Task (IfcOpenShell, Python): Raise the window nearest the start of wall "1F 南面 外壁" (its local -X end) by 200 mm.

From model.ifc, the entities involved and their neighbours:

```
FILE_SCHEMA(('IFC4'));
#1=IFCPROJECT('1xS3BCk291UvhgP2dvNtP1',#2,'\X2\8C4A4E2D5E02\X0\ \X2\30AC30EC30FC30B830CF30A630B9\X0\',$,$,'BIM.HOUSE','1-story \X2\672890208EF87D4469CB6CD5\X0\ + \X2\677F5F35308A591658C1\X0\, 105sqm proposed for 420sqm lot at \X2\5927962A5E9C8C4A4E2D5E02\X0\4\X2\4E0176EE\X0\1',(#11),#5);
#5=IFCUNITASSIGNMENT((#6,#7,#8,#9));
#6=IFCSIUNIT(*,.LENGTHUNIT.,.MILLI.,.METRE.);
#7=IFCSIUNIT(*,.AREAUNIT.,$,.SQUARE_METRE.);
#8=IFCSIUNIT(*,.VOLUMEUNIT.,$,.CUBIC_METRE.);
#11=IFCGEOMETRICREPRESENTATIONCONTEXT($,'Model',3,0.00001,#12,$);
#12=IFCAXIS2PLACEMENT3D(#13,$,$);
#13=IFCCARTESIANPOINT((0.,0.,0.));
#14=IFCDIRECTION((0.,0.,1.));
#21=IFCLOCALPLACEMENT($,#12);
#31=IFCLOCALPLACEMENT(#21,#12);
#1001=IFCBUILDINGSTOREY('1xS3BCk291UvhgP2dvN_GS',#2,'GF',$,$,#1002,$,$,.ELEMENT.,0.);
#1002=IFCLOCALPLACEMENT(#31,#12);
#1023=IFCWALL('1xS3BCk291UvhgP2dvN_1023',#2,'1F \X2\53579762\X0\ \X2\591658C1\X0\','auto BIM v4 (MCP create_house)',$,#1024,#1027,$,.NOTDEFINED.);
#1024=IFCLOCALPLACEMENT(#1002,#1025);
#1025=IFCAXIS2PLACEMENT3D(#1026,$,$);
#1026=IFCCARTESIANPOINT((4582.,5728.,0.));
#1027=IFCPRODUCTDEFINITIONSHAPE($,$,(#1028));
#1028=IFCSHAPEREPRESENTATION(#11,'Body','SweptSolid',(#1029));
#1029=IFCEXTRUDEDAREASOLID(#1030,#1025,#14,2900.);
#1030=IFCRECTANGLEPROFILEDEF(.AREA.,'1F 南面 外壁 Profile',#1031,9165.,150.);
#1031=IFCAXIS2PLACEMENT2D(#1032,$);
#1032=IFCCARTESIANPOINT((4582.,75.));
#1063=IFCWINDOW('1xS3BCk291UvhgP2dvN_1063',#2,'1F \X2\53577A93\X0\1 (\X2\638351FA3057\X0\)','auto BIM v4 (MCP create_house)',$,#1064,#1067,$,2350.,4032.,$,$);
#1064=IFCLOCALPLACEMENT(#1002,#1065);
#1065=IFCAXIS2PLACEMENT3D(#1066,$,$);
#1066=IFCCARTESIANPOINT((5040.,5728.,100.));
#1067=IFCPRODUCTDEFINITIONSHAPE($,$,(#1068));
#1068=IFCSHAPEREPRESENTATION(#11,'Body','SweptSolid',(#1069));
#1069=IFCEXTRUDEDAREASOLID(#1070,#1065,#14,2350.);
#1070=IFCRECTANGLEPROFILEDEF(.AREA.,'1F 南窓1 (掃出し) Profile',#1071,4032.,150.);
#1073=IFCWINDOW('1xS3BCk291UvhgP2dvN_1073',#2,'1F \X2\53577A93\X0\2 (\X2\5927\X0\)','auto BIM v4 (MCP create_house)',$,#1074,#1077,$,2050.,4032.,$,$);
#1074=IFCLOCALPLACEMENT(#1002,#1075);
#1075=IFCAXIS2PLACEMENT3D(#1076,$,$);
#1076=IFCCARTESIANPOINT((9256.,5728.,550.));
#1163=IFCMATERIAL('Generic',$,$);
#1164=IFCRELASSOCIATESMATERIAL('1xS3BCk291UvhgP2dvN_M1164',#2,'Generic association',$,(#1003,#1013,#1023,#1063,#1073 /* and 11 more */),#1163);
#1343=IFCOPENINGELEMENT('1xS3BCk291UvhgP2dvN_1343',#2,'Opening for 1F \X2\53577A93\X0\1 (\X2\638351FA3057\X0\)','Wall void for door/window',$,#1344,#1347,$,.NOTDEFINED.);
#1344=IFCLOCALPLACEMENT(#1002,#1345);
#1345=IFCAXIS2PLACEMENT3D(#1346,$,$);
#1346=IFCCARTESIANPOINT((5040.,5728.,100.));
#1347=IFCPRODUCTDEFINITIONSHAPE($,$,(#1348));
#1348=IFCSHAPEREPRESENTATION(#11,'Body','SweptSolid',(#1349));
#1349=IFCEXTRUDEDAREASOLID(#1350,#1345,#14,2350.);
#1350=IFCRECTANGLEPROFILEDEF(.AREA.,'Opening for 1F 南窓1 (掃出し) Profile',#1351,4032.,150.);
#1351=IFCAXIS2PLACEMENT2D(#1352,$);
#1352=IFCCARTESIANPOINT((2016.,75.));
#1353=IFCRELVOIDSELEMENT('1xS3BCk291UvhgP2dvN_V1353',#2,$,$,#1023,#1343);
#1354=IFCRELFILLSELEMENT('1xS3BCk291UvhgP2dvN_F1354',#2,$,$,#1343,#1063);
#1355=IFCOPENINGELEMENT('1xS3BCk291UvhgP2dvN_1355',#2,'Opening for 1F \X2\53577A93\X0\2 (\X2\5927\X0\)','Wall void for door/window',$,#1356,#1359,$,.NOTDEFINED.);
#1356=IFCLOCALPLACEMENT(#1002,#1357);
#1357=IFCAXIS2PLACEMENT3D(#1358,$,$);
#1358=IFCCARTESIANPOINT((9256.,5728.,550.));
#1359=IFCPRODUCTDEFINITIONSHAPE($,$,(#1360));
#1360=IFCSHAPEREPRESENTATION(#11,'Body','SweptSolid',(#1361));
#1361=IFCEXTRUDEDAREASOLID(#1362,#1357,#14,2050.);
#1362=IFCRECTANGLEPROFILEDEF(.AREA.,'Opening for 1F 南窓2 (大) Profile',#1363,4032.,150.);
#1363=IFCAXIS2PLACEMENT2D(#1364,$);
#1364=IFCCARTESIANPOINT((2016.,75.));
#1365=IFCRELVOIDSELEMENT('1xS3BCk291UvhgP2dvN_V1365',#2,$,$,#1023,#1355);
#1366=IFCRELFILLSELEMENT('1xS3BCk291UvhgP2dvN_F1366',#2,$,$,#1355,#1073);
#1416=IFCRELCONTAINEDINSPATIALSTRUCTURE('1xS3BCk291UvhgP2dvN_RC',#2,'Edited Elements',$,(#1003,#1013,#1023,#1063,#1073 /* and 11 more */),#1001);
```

```python
import numpy as np
import ifcopenshell
import ifcopenshell.api.geometry
import ifcopenshell.util.placement
import ifcopenshell.util.unit

model = ifcopenshell.open("model.ifc")
unit_scale = ifcopenshell.util.unit.calculate_unit_scale(model)

window = model.by_id(1063)
opening = window.FillsVoids[0].RelatingOpeningElement
dz = 0.2 / unit_scale

shift = np.array([0.0, 0.0, dz])
# The window is not placed relative to its opening, so move both.
for product in (opening, window):
    matrix = ifcopenshell.util.placement.get_local_placement(product.ObjectPlacement)
    matrix[:3, 3] += shift
    ifcopenshell.api.geometry.edit_object_placement(model, product=product, matrix=matrix, is_si=False)

print(f"moved by {dz * unit_scale:+.3f} m")

model.write("model_rev.ifc")
```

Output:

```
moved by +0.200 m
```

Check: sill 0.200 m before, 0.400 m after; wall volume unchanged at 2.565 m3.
